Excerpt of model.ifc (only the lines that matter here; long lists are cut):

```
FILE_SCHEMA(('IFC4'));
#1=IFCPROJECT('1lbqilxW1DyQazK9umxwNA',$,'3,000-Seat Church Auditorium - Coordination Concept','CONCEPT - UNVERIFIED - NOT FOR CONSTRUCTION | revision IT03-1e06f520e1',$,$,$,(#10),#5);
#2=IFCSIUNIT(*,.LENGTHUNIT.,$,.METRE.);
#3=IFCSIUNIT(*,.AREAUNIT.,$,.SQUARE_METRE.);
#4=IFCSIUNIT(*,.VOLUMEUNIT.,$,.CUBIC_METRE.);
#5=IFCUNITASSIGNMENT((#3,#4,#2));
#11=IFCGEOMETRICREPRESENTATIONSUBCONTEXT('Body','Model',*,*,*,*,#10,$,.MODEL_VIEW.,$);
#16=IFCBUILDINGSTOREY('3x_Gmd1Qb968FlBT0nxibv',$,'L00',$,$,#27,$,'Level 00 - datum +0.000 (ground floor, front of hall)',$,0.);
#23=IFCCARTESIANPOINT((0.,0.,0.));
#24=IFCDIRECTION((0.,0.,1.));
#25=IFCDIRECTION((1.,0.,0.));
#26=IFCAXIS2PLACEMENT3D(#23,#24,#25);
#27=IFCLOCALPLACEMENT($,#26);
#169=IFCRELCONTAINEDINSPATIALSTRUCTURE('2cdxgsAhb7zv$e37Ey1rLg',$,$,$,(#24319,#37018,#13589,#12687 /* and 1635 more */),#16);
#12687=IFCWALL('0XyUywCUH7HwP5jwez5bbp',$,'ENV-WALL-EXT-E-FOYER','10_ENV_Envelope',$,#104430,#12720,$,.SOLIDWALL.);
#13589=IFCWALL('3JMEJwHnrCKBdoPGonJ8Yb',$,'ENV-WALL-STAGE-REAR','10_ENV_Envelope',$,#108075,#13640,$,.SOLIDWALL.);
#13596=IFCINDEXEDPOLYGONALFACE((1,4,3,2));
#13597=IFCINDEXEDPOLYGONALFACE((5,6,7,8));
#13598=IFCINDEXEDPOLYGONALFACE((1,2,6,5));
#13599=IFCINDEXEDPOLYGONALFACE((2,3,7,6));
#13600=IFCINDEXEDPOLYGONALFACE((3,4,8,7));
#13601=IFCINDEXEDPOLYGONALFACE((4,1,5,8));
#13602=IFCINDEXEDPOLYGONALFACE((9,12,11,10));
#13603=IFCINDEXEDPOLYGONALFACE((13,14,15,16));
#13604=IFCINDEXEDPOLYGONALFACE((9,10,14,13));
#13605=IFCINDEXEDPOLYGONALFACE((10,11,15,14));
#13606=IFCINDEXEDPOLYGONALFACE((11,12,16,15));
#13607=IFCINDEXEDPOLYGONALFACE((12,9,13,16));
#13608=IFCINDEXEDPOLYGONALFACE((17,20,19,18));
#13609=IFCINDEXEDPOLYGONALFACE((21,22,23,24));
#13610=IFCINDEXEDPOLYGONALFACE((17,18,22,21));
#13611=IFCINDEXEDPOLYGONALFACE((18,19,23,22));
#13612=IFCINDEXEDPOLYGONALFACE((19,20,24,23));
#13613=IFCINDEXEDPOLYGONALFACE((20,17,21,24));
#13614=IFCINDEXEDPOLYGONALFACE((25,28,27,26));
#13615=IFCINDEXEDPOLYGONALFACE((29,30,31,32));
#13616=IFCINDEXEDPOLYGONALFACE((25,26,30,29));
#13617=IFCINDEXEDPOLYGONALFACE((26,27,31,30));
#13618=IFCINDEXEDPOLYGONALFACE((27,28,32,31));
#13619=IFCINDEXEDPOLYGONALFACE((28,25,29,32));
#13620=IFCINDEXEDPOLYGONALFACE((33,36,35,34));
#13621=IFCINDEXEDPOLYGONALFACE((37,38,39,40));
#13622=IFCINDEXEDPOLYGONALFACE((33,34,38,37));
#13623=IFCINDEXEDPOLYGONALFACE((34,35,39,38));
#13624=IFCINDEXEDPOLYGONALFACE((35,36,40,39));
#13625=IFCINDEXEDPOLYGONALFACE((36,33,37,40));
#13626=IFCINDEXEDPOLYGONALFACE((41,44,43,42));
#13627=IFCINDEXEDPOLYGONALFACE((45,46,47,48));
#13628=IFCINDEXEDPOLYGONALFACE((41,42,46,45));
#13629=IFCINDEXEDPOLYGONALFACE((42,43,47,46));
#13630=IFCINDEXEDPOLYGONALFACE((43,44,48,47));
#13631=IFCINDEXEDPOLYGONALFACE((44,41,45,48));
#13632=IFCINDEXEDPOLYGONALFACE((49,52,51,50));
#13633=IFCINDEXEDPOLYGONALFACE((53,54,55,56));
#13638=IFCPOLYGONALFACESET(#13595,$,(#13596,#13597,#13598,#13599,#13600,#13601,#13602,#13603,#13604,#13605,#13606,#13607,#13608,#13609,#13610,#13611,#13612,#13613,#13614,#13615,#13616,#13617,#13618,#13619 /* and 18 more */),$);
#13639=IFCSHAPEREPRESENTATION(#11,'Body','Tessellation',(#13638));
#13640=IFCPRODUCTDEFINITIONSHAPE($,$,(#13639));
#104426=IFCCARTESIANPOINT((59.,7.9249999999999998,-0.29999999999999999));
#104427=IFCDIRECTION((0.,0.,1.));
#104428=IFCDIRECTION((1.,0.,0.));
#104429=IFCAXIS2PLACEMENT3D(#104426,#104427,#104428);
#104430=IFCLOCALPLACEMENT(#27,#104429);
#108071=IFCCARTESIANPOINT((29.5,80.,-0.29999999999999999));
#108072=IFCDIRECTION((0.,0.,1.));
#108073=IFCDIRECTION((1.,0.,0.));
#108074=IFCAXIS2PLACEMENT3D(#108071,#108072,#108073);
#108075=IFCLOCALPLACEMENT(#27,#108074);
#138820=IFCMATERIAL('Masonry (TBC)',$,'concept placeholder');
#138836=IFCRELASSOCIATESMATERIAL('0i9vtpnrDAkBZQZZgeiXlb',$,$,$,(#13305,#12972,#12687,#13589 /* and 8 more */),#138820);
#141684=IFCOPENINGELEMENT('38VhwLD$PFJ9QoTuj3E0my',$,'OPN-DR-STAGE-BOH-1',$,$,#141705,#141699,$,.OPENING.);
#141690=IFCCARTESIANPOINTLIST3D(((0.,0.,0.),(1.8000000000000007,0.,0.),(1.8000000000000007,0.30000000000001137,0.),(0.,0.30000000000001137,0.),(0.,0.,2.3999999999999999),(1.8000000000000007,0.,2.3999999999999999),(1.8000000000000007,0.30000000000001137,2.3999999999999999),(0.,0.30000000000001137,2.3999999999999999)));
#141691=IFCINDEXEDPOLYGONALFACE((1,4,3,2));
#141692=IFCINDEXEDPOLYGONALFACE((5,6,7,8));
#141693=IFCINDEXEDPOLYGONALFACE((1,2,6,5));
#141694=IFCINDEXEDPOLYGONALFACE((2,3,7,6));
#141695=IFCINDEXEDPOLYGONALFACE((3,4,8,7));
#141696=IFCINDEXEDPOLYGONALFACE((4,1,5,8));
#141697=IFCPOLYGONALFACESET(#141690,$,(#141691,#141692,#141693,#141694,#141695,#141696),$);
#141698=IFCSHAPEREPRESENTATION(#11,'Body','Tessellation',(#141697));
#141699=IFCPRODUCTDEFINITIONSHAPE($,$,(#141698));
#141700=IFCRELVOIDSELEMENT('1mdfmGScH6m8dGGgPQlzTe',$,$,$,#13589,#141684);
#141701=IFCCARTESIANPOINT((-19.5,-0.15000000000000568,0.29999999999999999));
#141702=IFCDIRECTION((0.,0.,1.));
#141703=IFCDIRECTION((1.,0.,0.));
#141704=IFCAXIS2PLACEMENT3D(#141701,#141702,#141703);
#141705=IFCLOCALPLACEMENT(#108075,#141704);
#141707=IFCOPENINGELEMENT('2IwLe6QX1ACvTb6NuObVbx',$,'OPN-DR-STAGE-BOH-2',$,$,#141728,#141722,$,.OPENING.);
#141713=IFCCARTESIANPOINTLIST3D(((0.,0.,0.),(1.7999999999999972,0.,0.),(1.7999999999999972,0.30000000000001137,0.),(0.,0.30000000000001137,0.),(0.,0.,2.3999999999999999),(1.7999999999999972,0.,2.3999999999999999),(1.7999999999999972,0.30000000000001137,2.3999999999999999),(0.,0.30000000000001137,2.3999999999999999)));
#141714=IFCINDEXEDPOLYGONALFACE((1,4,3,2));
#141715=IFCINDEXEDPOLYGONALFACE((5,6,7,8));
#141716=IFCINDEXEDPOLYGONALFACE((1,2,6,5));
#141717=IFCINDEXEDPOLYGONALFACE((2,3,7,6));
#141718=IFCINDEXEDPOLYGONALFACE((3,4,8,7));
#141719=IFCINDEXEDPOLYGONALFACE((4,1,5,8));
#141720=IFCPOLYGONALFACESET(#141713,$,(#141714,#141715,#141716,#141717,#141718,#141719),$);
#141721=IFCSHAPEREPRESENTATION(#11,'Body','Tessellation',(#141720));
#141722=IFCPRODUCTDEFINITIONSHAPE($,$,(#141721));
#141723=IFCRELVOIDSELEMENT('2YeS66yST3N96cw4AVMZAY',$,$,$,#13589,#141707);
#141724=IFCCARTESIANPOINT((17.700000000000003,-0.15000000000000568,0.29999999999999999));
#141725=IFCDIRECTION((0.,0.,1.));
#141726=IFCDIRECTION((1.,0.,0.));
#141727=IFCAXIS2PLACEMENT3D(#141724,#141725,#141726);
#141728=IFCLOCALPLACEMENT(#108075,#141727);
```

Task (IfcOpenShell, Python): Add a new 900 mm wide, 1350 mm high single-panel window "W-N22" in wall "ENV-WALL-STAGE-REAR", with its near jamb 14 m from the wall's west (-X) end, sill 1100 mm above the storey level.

```python
import numpy as np
import ifcopenshell
import ifcopenshell.api.feature
import ifcopenshell.api.geometry
import ifcopenshell.api.root
import ifcopenshell.api.spatial
import ifcopenshell.geom
import ifcopenshell.util.element
import ifcopenshell.util.placement
import ifcopenshell.util.representation
import ifcopenshell.util.shape
import ifcopenshell.util.unit

model = ifcopenshell.open("model.ifc")
unit_scale = ifcopenshell.util.unit.calculate_unit_scale(model)
settings = ifcopenshell.geom.settings()


def volume(element):
    """Net volume in cubic metres, openings subtracted."""
    shape = ifcopenshell.geom.create_shape(settings, element)
    return ifcopenshell.util.shape.get_volume(shape.geometry)


wall = model.by_guid("3JMEJwHnrCKBdoPGonJ8Yb")
storey = ifcopenshell.util.element.get_container(wall, ifc_class="IfcBuildingStorey")
context = ifcopenshell.util.representation.get_context(model, "Model", "Body", "MODEL_VIEW")
before = volume(wall)

width, height, from_end, sill = 0.9, 1.35, 14, 1.1  # metres

# The wall runs along its own X axis, and the end named is its -X end.
wall_shape = ifcopenshell.geom.create_shape(settings, wall)
x, y, z = ifcopenshell.util.shape.get_vertices(wall_shape.geometry).T
start = x.min() + from_end
face, thickness = float(y.min()), float(y.max() - y.min())
wall_matrix = ifcopenshell.util.placement.get_local_placement(wall.ObjectPlacement)
level = ifcopenshell.util.placement.get_local_placement(storey.ObjectPlacement)[2, 3]


def in_wall(x, y):
    """Placement at x, y metres in the wall's axes, at sill height."""
    matrix = wall_matrix.copy()
    matrix[:, 3] = wall_matrix @ np.array([x / unit_scale, y / unit_scale, 0.0, 1.0])
    matrix[2, 3] = level + sill / unit_scale
    return matrix


# Opening: a box that overshoots both wall faces by 50 mm.
opening = ifcopenshell.api.root.create_entity(model, ifc_class="IfcOpeningElement", predefined_type="OPENING")
box = ifcopenshell.api.geometry.add_wall_representation(
    model, context=context, length=width, height=height, thickness=thickness + 0.1
)
ifcopenshell.api.geometry.assign_representation(model, product=opening, representation=box)
ifcopenshell.api.geometry.edit_object_placement(model, product=opening, matrix=in_wall(start, face - 0.05), is_si=False)
ifcopenshell.api.feature.add_feature(model, feature=opening, element=wall)

window = ifcopenshell.api.root.create_entity(model, ifc_class="IfcWindow", name="W-N22", predefined_type="WINDOW")
window.OverallWidth, window.OverallHeight = width / unit_scale, height / unit_scale
window.PartitioningType = "SINGLE_PANEL"
body = ifcopenshell.api.geometry.add_window_representation(
    model,
    context=context,
    overall_width=window.OverallWidth,
    overall_height=window.OverallHeight,
    partition_type="SINGLE_PANEL",
)
ifcopenshell.api.geometry.assign_representation(model, product=window, representation=body)
ifcopenshell.api.spatial.assign_container(model, products=[window], relating_structure=storey)
ifcopenshell.api.feature.add_filling(model, opening=opening, element=window)

# Centre the window in the wall's thickness.
ifcopenshell.api.geometry.edit_object_placement(model, product=window, matrix=in_wall(start, face), is_si=False)
window_shape = ifcopenshell.geom.create_shape(settings, window)
depth = ifcopenshell.util.shape.get_vertices(window_shape.geometry)[:, 1]
offset = face + thickness / 2 - (depth.min() + depth.max()) / 2
ifcopenshell.api.geometry.edit_object_placement(model, product=window, matrix=in_wall(start, offset), is_si=False)

after = volume(wall)

print(f"wall volume {before:.3f} -> {after:.3f} m3")

model.write("model_updated.ifc")
```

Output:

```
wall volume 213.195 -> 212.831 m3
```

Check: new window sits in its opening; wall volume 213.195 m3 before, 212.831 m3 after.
